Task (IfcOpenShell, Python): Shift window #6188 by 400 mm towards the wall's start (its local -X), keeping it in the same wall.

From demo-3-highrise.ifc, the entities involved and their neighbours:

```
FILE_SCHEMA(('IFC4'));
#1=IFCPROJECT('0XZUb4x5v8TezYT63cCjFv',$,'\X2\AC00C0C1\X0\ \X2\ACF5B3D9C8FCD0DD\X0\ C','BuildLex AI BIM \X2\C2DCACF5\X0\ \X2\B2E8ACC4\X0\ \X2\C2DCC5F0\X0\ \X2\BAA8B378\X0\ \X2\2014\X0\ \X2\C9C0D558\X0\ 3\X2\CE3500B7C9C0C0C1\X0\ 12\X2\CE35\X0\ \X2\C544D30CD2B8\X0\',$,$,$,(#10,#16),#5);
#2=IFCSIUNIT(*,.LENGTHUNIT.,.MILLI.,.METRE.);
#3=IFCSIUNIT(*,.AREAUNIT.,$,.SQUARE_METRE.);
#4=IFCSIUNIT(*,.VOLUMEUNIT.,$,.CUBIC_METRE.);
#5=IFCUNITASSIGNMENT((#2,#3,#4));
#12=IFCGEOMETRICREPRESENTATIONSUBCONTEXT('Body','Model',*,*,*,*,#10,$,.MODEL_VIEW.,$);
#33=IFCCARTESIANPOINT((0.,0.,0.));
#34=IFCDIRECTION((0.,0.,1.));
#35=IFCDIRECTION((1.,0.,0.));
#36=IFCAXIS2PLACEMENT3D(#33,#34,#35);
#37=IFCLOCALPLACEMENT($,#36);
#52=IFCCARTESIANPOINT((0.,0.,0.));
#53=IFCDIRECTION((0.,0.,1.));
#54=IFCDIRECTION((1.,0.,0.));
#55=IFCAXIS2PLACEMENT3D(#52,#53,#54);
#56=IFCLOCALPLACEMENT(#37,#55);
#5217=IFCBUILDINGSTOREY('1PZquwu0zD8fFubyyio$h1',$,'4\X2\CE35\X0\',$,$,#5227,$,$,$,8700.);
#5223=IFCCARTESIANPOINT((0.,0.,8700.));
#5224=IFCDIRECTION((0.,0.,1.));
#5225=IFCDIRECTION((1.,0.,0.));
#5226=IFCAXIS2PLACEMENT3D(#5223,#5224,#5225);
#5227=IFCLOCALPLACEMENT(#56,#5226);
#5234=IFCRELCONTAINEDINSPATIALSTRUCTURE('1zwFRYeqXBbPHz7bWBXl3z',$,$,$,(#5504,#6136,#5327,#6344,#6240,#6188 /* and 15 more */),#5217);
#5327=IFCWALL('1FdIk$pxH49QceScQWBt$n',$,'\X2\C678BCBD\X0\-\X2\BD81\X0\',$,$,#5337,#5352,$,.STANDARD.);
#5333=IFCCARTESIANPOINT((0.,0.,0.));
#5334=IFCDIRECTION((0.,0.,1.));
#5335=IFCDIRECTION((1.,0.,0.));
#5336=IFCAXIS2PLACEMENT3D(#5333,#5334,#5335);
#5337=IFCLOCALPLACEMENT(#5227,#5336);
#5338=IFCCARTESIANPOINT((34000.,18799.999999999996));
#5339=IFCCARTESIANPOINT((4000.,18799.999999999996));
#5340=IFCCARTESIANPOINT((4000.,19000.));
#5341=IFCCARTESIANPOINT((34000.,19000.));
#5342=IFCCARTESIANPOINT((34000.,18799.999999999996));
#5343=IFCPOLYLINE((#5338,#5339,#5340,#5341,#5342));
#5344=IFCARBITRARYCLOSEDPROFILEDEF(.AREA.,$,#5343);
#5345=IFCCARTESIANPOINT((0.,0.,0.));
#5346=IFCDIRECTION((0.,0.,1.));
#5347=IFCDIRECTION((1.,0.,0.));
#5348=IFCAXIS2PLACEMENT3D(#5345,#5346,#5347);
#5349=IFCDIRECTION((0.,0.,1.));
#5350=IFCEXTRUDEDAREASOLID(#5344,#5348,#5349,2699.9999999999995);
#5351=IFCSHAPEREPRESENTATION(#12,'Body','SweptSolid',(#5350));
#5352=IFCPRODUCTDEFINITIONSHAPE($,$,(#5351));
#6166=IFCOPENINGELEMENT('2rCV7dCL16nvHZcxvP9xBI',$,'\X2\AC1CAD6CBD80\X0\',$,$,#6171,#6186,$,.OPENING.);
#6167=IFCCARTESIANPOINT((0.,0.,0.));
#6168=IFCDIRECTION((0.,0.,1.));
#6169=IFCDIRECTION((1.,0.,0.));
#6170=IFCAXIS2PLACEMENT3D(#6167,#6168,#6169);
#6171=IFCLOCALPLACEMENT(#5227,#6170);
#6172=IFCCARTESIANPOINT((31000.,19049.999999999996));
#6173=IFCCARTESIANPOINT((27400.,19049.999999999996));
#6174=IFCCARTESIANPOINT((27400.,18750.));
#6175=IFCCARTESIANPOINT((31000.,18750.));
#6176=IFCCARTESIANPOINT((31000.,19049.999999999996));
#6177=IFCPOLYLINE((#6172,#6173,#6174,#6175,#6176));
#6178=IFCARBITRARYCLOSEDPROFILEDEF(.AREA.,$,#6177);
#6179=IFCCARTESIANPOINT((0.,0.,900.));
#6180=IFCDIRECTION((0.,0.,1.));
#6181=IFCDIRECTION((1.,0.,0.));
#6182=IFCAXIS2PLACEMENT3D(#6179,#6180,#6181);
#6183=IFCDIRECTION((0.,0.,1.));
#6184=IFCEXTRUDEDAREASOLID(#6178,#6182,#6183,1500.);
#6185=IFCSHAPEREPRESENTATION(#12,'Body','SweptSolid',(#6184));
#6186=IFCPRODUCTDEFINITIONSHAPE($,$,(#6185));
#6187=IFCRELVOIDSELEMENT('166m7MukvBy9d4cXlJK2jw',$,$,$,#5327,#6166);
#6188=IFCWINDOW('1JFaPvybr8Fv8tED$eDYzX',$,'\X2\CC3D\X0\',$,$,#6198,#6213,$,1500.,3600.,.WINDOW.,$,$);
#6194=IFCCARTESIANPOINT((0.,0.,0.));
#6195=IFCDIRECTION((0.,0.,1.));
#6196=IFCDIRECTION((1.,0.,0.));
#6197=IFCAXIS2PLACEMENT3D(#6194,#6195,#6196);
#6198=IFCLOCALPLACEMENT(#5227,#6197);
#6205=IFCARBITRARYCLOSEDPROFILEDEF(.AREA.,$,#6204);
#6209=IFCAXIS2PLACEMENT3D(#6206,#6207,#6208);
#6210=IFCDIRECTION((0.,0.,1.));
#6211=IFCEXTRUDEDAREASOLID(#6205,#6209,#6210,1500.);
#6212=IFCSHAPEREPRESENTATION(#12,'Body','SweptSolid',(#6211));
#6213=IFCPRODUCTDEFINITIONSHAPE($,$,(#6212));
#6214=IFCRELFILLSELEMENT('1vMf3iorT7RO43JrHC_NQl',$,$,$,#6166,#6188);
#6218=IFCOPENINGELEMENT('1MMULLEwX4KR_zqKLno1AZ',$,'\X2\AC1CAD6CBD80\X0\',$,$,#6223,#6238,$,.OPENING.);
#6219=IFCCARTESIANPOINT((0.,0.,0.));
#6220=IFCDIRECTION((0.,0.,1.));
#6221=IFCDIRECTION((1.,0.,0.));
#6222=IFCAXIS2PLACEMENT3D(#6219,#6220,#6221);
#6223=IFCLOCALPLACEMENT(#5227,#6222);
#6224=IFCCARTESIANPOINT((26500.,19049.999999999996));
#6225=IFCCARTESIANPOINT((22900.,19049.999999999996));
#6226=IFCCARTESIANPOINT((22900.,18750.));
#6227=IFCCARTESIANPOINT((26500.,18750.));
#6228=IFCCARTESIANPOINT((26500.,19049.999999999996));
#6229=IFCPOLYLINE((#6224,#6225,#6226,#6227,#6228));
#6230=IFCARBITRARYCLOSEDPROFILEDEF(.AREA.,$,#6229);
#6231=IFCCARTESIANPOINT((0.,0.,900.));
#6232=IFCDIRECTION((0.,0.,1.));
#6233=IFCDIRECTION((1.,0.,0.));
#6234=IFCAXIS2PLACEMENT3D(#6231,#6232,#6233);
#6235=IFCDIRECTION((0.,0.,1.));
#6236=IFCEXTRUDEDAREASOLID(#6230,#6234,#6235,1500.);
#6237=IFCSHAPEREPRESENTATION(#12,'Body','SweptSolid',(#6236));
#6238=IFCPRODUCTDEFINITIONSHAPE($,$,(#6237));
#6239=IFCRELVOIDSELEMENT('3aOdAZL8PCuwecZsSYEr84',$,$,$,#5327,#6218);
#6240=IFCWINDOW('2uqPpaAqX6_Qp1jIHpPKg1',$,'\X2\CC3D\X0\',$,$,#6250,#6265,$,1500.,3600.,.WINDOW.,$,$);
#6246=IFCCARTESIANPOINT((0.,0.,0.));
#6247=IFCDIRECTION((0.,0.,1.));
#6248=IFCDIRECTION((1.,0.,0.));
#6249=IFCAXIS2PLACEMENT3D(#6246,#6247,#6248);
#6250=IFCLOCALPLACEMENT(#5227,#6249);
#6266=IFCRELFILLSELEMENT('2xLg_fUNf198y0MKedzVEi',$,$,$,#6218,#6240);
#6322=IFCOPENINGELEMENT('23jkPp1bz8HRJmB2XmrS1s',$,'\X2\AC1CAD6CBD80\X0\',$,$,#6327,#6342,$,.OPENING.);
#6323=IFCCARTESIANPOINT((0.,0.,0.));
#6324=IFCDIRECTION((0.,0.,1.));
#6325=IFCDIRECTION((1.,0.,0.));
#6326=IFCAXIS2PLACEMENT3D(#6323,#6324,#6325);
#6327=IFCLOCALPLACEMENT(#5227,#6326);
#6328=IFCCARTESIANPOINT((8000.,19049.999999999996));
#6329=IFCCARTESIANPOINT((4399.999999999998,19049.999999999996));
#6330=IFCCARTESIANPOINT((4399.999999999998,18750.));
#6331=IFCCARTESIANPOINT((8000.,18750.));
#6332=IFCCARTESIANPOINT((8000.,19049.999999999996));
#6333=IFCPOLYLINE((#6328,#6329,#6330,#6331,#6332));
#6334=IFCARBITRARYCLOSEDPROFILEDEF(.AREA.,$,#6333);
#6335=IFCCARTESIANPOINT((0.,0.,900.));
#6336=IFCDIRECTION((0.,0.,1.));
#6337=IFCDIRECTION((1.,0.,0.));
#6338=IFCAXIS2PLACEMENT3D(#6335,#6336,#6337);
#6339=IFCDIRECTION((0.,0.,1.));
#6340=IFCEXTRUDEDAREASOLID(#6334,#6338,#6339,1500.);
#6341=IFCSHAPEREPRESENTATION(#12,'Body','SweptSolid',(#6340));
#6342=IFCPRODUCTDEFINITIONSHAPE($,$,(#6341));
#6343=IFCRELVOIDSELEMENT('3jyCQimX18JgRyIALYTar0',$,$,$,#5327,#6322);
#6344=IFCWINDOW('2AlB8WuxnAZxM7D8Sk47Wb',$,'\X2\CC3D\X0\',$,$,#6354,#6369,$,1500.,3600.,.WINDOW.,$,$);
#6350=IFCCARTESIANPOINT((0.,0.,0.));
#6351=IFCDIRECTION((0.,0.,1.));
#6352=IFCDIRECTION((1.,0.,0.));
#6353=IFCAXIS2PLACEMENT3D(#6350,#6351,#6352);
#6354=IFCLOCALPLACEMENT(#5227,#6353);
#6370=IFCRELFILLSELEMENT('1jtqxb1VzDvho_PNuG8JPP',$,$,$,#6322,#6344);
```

```python
import ifcopenshell
import ifcopenshell.api.geometry
import ifcopenshell.util.placement

model = ifcopenshell.open("demo-3-highrise.ifc")

window = model.by_id(6188)
opening = window.FillsVoids[0].RelatingOpeningElement
wall = opening.VoidsElements[0].RelatingBuildingElement

wall_matrix = ifcopenshell.util.placement.get_local_placement(wall.ObjectPlacement)
shift = wall_matrix[:3, 0] * -400.0
before = ifcopenshell.util.placement.get_local_placement(window.ObjectPlacement)[:3, 3].copy()

# The window is not placed relative to its opening, so move both.
for product in (opening, window):
    matrix = ifcopenshell.util.placement.get_local_placement(product.ObjectPlacement)
    matrix[:3, 3] += shift
    ifcopenshell.api.geometry.edit_object_placement(model, product=product, matrix=matrix, is_si=False)

after = ifcopenshell.util.placement.get_local_placement(window.ObjectPlacement)[:3, 3]
print("window moved by", (after - before).round(3) + 0.0)

model.write("demo-3-highrise_updated.ifc")
```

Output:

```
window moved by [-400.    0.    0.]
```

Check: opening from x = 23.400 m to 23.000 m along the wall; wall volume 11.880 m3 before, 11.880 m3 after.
